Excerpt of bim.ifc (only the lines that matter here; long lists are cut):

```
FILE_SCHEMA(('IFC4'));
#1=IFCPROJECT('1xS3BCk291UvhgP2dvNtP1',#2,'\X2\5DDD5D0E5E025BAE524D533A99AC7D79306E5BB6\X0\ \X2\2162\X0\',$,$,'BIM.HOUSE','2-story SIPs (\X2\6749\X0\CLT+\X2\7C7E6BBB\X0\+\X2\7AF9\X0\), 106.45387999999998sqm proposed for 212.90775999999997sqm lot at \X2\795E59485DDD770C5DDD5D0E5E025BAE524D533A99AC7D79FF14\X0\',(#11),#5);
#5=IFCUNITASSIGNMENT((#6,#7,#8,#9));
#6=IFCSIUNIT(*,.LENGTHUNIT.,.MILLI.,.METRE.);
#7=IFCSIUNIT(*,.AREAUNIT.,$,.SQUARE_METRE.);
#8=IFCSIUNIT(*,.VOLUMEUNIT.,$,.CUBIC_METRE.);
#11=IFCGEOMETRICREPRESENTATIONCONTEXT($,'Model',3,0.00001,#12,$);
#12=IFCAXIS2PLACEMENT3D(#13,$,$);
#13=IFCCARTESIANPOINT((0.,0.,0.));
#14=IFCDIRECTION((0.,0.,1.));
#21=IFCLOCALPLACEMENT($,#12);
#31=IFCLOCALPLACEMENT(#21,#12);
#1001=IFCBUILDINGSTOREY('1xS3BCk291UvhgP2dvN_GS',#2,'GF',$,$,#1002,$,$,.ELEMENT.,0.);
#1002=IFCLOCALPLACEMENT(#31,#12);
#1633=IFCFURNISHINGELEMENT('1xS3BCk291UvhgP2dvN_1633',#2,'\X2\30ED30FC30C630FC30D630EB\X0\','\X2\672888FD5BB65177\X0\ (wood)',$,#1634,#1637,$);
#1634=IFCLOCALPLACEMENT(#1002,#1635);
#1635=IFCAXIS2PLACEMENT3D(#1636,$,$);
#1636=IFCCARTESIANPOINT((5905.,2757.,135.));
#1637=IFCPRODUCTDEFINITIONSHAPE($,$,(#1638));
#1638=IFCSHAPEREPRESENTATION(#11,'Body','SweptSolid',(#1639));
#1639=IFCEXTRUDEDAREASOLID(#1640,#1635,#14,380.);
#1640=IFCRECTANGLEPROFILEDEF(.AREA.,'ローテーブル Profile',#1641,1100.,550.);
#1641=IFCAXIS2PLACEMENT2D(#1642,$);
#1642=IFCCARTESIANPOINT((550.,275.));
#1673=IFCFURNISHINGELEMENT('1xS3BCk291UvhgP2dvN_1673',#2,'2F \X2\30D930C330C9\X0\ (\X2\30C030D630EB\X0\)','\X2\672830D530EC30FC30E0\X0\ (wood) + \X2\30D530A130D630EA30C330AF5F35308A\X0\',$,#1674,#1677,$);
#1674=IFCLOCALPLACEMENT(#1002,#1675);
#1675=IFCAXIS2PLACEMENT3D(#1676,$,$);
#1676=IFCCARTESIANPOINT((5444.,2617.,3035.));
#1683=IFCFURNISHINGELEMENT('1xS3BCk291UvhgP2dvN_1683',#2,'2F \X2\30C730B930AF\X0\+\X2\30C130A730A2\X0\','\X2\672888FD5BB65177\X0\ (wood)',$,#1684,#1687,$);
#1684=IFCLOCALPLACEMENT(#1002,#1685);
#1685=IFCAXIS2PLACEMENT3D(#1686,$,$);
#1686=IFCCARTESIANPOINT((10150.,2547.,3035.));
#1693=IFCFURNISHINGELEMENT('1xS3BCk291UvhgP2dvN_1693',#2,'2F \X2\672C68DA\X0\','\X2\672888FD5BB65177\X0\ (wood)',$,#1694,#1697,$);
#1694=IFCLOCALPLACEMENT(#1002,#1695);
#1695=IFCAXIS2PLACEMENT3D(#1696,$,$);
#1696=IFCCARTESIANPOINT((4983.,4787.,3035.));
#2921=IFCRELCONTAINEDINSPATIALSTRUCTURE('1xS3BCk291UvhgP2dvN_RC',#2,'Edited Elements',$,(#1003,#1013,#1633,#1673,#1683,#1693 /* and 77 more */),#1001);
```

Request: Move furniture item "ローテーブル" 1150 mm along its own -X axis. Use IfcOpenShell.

```python
import ifcopenshell
import ifcopenshell.api.geometry
import ifcopenshell.util.placement
import ifcopenshell.util.unit

model = ifcopenshell.open("bim.ifc")
unit_scale = ifcopenshell.util.unit.calculate_unit_scale(model)

item = model.by_guid("1xS3BCk291UvhgP2dvN_1633")
matrix = ifcopenshell.util.placement.get_local_placement(item.ObjectPlacement)
matrix[:3, 3] -= matrix[:3, 0] * 1.15 / unit_scale
ifcopenshell.api.geometry.edit_object_placement(model, product=item, matrix=matrix, is_si=False)

print(ifcopenshell.util.placement.get_local_placement(item.ObjectPlacement).round(3) + 0.0)

model.write("bim_rev.ifc")
```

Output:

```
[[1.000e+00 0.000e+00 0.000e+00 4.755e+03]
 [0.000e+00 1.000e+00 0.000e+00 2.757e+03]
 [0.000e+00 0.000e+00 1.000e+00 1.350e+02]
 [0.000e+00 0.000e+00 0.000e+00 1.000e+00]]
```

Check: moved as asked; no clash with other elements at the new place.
